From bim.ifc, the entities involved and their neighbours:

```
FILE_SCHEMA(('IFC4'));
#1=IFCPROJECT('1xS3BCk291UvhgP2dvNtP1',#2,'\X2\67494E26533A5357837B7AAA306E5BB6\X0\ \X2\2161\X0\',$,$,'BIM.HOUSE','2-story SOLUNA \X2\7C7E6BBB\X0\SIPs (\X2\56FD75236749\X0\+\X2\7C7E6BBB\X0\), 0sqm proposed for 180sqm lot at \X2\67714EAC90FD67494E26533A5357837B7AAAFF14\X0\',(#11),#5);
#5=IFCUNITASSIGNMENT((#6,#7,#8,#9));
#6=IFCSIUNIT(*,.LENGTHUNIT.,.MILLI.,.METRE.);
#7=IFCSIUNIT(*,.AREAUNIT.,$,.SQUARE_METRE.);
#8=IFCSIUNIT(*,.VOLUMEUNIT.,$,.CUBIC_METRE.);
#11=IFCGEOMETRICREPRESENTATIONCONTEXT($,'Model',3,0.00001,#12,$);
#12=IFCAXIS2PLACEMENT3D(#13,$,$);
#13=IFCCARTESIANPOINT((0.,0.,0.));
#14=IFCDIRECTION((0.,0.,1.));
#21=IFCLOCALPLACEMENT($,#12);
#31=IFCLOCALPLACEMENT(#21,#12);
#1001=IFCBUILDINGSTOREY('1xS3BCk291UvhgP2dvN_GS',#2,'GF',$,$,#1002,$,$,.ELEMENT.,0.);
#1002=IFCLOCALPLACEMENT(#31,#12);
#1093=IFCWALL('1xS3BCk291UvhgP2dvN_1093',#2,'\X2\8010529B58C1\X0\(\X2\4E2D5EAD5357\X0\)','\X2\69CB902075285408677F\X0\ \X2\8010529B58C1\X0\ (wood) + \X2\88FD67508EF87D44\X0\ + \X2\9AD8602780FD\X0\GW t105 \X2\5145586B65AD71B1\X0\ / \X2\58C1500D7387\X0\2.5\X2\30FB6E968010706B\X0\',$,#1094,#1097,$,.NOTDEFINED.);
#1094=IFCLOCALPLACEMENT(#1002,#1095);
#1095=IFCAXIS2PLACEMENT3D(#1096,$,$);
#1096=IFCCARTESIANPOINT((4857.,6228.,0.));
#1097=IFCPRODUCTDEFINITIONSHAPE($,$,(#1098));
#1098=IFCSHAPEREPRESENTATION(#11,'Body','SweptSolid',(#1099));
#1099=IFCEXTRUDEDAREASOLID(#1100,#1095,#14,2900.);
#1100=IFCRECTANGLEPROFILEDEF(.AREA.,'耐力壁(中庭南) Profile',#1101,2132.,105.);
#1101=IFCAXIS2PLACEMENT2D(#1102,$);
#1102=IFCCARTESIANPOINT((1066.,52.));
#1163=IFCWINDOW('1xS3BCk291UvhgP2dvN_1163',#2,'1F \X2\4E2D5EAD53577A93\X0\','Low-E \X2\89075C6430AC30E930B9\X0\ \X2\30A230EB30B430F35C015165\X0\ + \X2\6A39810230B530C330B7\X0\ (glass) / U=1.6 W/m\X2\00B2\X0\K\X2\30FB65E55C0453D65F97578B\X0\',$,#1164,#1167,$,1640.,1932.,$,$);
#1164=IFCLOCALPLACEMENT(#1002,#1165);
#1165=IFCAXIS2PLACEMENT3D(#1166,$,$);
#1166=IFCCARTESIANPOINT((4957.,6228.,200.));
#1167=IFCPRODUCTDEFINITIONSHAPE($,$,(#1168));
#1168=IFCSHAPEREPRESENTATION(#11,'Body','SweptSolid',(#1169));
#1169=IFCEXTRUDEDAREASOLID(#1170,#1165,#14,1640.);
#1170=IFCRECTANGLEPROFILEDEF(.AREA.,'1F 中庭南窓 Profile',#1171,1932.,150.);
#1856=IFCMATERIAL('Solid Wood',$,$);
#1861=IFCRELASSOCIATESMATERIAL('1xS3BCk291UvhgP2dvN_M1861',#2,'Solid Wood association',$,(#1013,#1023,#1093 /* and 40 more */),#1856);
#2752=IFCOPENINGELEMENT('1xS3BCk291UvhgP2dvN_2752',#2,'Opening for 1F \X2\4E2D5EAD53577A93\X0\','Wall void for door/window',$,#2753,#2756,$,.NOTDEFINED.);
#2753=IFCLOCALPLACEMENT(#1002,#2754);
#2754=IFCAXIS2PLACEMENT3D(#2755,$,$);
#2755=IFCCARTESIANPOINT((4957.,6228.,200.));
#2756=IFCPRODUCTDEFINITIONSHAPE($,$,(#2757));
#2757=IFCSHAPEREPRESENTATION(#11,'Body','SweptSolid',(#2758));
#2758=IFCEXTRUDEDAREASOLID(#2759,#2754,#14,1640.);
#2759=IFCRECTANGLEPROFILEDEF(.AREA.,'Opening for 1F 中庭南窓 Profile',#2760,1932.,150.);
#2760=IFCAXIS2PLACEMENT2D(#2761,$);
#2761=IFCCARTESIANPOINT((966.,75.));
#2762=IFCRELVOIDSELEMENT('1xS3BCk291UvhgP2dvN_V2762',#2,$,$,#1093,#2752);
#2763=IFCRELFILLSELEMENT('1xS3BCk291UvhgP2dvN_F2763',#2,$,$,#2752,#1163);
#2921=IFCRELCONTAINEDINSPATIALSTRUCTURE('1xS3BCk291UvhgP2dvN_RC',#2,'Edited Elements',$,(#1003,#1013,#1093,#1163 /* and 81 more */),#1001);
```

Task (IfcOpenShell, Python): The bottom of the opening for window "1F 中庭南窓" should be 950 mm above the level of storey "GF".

```python
import numpy as np
import ifcopenshell
import ifcopenshell.api.geometry
import ifcopenshell.geom
import ifcopenshell.util.element
import ifcopenshell.util.placement
import ifcopenshell.util.shape
import ifcopenshell.util.unit

model = ifcopenshell.open("bim.ifc")
unit_scale = ifcopenshell.util.unit.calculate_unit_scale(model)

window = model.by_id(1163)
opening = window.FillsVoids[0].RelatingOpeningElement
storey = ifcopenshell.util.element.get_container(window, ifc_class="IfcBuildingStorey")
level = ifcopenshell.util.placement.get_local_placement(storey.ObjectPlacement)[2, 3]

# The opening's origin need not be at the sill, so measure its lowest point.
shape = ifcopenshell.geom.create_shape(ifcopenshell.geom.settings(), opening)
bottom = ifcopenshell.util.shape.get_shape_bottom_elevation(shape, shape.geometry) / unit_scale
dz = level + 0.95 / unit_scale - bottom

shift = np.array([0.0, 0.0, dz])
# The window is not placed relative to its opening, so move both.
for product in (opening, window):
    matrix = ifcopenshell.util.placement.get_local_placement(product.ObjectPlacement)
    matrix[:3, 3] += shift
    ifcopenshell.api.geometry.edit_object_placement(model, product=product, matrix=matrix, is_si=False)

print(f"moved by {dz * unit_scale:+.3f} m")

model.write("bim_v2.ifc")
```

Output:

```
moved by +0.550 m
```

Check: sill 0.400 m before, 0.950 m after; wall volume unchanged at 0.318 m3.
